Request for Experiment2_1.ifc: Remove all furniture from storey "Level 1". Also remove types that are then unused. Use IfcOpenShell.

First a look at what the model holds.

```python
import ifcopenshell
import ifcopenshell.util.element

model = ifcopenshell.open("Experiment2_1.ifc")
print(model.schema)
storey = next(s for s in model.by_type("IfcBuildingStorey") if s.Name == "Level 1")
furniture = [e for e in ifcopenshell.util.element.get_decomposition(storey) if e.is_a("IfcFurnishingElement")]
seen = {}
for e in furniture:
    element_type = ifcopenshell.util.element.get_type(e)
    name = element_type.Name if element_type not in (None, e) else None
    seen[name] = seen.get(name, 0) + 1
for name, count in sorted(seen.items(), key=str):
    print(count, "x", name)
```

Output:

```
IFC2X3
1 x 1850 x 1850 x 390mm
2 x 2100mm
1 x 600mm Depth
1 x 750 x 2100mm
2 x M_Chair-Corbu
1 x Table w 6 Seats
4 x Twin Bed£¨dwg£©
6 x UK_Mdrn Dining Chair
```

```python
import ifcopenshell
import ifcopenshell.api.root
import ifcopenshell.util.element

model = ifcopenshell.open("Experiment2_1.ifc")

storey = next(s for s in model.by_type("IfcBuildingStorey") if s.Name == "Level 1")
furniture = [e for e in ifcopenshell.util.element.get_decomposition(storey) if e.is_a("IfcFurnishingElement")]
types = {ifcopenshell.util.element.get_type(e) for e in furniture} - {None, *furniture}

for e in furniture:
    ifcopenshell.api.root.remove_product(model, product=e)
print(len(furniture), "removed")

unused = [t for t in types if not ifcopenshell.util.element.get_types(t)]
for t in unused:
    ifcopenshell.api.root.remove_product(model, product=t)
print(len(unused), "unused types removed")

model.write("Experiment2_1-out.ifc")
```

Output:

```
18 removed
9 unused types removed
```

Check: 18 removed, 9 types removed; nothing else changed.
